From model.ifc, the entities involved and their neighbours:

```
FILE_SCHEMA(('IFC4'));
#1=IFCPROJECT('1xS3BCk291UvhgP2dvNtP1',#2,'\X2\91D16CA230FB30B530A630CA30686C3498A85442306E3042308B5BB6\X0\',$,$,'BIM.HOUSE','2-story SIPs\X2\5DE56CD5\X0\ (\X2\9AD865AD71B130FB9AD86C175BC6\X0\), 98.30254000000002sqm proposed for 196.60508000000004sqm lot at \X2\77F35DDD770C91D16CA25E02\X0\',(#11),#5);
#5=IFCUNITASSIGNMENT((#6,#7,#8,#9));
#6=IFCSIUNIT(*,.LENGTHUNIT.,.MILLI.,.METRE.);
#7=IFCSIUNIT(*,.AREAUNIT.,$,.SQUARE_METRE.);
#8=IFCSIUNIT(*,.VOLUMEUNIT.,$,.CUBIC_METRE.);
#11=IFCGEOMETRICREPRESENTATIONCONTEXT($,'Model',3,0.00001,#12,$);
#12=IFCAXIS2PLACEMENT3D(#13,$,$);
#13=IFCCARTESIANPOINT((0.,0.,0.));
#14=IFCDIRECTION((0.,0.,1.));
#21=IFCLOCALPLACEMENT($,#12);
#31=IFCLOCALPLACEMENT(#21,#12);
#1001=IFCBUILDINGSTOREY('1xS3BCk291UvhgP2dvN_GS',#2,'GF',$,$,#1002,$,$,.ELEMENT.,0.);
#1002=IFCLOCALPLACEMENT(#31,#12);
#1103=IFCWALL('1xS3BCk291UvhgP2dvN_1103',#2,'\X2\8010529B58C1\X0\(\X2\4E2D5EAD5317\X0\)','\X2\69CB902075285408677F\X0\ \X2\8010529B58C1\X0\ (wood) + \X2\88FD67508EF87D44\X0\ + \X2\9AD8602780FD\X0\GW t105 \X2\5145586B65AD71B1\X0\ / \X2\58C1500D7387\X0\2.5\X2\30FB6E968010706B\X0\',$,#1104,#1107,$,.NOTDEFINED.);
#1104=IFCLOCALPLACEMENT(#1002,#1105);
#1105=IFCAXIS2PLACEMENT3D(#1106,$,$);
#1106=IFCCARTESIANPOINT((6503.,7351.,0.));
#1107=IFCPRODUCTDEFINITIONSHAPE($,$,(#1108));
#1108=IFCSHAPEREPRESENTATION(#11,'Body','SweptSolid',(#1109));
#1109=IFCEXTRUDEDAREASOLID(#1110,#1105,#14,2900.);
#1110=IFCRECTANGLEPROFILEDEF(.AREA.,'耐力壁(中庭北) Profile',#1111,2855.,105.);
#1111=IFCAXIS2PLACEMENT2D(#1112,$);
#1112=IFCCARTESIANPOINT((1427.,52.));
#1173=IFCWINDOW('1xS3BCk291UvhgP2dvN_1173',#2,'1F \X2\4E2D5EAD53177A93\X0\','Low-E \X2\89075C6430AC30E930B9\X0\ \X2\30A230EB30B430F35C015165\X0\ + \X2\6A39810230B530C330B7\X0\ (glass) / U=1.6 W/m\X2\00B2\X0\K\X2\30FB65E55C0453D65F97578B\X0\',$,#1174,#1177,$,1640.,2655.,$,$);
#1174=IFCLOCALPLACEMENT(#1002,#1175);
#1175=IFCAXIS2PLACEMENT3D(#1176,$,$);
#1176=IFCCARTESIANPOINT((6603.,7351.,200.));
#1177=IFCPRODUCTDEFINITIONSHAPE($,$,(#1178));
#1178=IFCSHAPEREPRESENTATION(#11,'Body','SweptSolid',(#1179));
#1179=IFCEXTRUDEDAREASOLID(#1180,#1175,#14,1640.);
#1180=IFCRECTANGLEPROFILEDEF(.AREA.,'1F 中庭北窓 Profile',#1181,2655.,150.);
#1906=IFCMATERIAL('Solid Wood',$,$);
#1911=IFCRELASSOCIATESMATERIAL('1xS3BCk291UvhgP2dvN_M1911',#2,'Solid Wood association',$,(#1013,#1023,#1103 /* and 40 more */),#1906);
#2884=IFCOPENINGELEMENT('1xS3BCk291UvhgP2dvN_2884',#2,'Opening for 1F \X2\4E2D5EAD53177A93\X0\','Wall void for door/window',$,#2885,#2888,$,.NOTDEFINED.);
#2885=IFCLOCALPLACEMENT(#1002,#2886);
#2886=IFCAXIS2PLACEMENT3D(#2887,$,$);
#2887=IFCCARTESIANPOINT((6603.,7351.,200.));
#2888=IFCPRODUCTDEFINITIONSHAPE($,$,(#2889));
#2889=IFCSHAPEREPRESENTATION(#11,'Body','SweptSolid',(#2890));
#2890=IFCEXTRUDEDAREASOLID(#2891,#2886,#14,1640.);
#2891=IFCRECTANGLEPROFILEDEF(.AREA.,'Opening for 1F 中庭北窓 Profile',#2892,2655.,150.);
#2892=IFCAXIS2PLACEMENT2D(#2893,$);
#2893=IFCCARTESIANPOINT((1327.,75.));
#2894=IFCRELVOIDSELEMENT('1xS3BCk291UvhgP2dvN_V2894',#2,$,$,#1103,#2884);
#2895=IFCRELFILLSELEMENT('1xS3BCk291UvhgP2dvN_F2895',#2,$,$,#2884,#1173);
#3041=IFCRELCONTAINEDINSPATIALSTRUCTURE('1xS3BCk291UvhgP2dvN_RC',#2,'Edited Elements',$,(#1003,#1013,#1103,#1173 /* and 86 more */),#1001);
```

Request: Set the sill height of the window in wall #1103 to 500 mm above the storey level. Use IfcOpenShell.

```python
import numpy as np
import ifcopenshell
import ifcopenshell.api.geometry
import ifcopenshell.geom
import ifcopenshell.util.element
import ifcopenshell.util.placement
import ifcopenshell.util.shape
import ifcopenshell.util.unit

model = ifcopenshell.open("model.ifc")
unit_scale = ifcopenshell.util.unit.calculate_unit_scale(model)

window = model.by_guid("1xS3BCk291UvhgP2dvN_1173")
opening = window.FillsVoids[0].RelatingOpeningElement
storey = ifcopenshell.util.element.get_container(window, ifc_class="IfcBuildingStorey")
level = ifcopenshell.util.placement.get_local_placement(storey.ObjectPlacement)[2, 3]

# The opening's origin need not be at the sill, so measure its lowest point.
shape = ifcopenshell.geom.create_shape(ifcopenshell.geom.settings(), opening)
bottom = ifcopenshell.util.shape.get_shape_bottom_elevation(shape, shape.geometry) / unit_scale
dz = level + 500.0 - bottom

shift = np.array([0.0, 0.0, dz])
# The window is not placed relative to its opening, so move both.
for product in (opening, window):
    matrix = ifcopenshell.util.placement.get_local_placement(product.ObjectPlacement)
    matrix[:3, 3] += shift
    ifcopenshell.api.geometry.edit_object_placement(model, product=product, matrix=matrix, is_si=False)

print(f"moved by {dz * unit_scale:+.3f} m")

model.write("model_updated.ifc")
```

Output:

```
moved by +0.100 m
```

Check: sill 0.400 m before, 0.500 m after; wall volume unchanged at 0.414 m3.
